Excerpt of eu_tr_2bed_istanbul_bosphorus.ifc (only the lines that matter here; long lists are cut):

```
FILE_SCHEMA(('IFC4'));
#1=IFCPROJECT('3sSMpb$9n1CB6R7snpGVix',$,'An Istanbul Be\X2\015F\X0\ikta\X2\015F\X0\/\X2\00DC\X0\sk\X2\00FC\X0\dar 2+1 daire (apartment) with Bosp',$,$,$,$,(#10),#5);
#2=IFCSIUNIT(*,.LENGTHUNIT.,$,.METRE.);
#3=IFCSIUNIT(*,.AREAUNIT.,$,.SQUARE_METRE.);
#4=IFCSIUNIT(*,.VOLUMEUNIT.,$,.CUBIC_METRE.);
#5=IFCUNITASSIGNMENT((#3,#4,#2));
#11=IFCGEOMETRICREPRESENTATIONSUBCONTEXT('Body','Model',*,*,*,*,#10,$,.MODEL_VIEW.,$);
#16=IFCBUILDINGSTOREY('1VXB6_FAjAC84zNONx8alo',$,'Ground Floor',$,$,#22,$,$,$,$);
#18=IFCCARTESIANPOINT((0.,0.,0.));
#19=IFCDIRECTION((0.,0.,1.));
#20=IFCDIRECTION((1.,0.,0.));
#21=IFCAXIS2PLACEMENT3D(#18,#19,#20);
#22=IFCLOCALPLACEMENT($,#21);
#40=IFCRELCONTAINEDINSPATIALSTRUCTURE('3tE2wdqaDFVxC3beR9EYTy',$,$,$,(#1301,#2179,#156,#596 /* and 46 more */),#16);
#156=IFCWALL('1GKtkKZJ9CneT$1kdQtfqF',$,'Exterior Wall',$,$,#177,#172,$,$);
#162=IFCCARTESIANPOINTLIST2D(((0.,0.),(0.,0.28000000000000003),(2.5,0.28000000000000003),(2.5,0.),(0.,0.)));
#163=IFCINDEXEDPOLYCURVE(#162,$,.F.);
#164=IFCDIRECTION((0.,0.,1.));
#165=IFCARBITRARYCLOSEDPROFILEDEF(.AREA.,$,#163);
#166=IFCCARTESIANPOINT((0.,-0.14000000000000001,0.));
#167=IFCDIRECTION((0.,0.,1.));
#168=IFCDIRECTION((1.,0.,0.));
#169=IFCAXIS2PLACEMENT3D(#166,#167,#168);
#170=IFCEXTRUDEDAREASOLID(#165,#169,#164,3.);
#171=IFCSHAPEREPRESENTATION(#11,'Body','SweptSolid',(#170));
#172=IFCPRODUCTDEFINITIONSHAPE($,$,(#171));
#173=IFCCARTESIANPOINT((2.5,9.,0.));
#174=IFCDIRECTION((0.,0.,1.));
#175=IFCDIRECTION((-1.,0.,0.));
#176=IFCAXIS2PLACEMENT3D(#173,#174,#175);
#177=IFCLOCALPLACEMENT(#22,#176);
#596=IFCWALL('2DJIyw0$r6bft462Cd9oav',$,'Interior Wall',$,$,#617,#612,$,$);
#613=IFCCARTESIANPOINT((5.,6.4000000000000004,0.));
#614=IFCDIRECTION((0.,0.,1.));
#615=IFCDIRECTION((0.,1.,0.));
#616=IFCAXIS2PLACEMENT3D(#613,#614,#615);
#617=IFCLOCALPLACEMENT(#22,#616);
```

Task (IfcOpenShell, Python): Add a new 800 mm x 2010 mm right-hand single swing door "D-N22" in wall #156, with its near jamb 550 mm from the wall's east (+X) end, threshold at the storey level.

```python
import numpy as np
import ifcopenshell
import ifcopenshell.api.feature
import ifcopenshell.api.geometry
import ifcopenshell.api.root
import ifcopenshell.api.spatial
import ifcopenshell.geom
import ifcopenshell.util.element
import ifcopenshell.util.placement
import ifcopenshell.util.representation
import ifcopenshell.util.shape
import ifcopenshell.util.unit

model = ifcopenshell.open("eu_tr_2bed_istanbul_bosphorus.ifc")
unit_scale = ifcopenshell.util.unit.calculate_unit_scale(model)
settings = ifcopenshell.geom.settings()


def volume(element):
    """Net volume in cubic metres, openings subtracted."""
    shape = ifcopenshell.geom.create_shape(settings, element)
    return ifcopenshell.util.shape.get_volume(shape.geometry)


wall = model.by_id(156)
storey = ifcopenshell.util.element.get_container(wall, ifc_class="IfcBuildingStorey")
context = ifcopenshell.util.representation.get_context(model, "Model", "Body", "MODEL_VIEW")
before = volume(wall)

width, height, from_end, sill = 0.8, 2.01, 0.55, 0.0  # metres

# The wall runs along its own X axis, and the end named is its -X end.
wall_shape = ifcopenshell.geom.create_shape(settings, wall)
x, y, z = ifcopenshell.util.shape.get_vertices(wall_shape.geometry).T
start = x.min() + from_end
face, thickness = float(y.min()), float(y.max() - y.min())
wall_matrix = ifcopenshell.util.placement.get_local_placement(wall.ObjectPlacement)
level = ifcopenshell.util.placement.get_local_placement(storey.ObjectPlacement)[2, 3]


def in_wall(x, y):
    """Placement at x, y metres in the wall's axes, at sill height."""
    matrix = wall_matrix.copy()
    matrix[:, 3] = wall_matrix @ np.array([x / unit_scale, y / unit_scale, 0.0, 1.0])
    matrix[2, 3] = level + sill / unit_scale
    return matrix


# Opening: a box that overshoots both wall faces by 50 mm.
opening = ifcopenshell.api.root.create_entity(model, ifc_class="IfcOpeningElement", predefined_type="OPENING")
box = ifcopenshell.api.geometry.add_wall_representation(
    model, context=context, length=width, height=height, thickness=thickness + 0.1
)
ifcopenshell.api.geometry.assign_representation(model, product=opening, representation=box)
ifcopenshell.api.geometry.edit_object_placement(model, product=opening, matrix=in_wall(start, face - 0.05), is_si=False)
ifcopenshell.api.feature.add_feature(model, feature=opening, element=wall)

door = ifcopenshell.api.root.create_entity(model, ifc_class="IfcDoor", name="D-N22", predefined_type="DOOR")
door.OverallWidth, door.OverallHeight = width / unit_scale, height / unit_scale
door.OperationType = "SINGLE_SWING_RIGHT"
body = ifcopenshell.api.geometry.add_door_representation(
    model,
    context=context,
    overall_width=door.OverallWidth,
    overall_height=door.OverallHeight,
    operation_type="SINGLE_SWING_RIGHT",
    lining_properties={"LiningDepth": thickness / unit_scale, "ThresholdDepth": thickness / unit_scale},
)
ifcopenshell.api.geometry.assign_representation(model, product=door, representation=body)
ifcopenshell.api.spatial.assign_container(model, products=[door], relating_structure=storey)
ifcopenshell.api.feature.add_filling(model, opening=opening, element=door)

# The lining spans the wall, so the door starts at the wall face.
ifcopenshell.api.geometry.edit_object_placement(model, product=door, matrix=in_wall(start, face), is_si=False)

after = volume(wall)

print(f"wall volume {before:.3f} -> {after:.3f} m3")

model.write("eu_tr_2bed_istanbul_bosphorus_updated.ifc")
```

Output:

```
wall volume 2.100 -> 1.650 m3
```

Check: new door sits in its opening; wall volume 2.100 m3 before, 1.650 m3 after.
